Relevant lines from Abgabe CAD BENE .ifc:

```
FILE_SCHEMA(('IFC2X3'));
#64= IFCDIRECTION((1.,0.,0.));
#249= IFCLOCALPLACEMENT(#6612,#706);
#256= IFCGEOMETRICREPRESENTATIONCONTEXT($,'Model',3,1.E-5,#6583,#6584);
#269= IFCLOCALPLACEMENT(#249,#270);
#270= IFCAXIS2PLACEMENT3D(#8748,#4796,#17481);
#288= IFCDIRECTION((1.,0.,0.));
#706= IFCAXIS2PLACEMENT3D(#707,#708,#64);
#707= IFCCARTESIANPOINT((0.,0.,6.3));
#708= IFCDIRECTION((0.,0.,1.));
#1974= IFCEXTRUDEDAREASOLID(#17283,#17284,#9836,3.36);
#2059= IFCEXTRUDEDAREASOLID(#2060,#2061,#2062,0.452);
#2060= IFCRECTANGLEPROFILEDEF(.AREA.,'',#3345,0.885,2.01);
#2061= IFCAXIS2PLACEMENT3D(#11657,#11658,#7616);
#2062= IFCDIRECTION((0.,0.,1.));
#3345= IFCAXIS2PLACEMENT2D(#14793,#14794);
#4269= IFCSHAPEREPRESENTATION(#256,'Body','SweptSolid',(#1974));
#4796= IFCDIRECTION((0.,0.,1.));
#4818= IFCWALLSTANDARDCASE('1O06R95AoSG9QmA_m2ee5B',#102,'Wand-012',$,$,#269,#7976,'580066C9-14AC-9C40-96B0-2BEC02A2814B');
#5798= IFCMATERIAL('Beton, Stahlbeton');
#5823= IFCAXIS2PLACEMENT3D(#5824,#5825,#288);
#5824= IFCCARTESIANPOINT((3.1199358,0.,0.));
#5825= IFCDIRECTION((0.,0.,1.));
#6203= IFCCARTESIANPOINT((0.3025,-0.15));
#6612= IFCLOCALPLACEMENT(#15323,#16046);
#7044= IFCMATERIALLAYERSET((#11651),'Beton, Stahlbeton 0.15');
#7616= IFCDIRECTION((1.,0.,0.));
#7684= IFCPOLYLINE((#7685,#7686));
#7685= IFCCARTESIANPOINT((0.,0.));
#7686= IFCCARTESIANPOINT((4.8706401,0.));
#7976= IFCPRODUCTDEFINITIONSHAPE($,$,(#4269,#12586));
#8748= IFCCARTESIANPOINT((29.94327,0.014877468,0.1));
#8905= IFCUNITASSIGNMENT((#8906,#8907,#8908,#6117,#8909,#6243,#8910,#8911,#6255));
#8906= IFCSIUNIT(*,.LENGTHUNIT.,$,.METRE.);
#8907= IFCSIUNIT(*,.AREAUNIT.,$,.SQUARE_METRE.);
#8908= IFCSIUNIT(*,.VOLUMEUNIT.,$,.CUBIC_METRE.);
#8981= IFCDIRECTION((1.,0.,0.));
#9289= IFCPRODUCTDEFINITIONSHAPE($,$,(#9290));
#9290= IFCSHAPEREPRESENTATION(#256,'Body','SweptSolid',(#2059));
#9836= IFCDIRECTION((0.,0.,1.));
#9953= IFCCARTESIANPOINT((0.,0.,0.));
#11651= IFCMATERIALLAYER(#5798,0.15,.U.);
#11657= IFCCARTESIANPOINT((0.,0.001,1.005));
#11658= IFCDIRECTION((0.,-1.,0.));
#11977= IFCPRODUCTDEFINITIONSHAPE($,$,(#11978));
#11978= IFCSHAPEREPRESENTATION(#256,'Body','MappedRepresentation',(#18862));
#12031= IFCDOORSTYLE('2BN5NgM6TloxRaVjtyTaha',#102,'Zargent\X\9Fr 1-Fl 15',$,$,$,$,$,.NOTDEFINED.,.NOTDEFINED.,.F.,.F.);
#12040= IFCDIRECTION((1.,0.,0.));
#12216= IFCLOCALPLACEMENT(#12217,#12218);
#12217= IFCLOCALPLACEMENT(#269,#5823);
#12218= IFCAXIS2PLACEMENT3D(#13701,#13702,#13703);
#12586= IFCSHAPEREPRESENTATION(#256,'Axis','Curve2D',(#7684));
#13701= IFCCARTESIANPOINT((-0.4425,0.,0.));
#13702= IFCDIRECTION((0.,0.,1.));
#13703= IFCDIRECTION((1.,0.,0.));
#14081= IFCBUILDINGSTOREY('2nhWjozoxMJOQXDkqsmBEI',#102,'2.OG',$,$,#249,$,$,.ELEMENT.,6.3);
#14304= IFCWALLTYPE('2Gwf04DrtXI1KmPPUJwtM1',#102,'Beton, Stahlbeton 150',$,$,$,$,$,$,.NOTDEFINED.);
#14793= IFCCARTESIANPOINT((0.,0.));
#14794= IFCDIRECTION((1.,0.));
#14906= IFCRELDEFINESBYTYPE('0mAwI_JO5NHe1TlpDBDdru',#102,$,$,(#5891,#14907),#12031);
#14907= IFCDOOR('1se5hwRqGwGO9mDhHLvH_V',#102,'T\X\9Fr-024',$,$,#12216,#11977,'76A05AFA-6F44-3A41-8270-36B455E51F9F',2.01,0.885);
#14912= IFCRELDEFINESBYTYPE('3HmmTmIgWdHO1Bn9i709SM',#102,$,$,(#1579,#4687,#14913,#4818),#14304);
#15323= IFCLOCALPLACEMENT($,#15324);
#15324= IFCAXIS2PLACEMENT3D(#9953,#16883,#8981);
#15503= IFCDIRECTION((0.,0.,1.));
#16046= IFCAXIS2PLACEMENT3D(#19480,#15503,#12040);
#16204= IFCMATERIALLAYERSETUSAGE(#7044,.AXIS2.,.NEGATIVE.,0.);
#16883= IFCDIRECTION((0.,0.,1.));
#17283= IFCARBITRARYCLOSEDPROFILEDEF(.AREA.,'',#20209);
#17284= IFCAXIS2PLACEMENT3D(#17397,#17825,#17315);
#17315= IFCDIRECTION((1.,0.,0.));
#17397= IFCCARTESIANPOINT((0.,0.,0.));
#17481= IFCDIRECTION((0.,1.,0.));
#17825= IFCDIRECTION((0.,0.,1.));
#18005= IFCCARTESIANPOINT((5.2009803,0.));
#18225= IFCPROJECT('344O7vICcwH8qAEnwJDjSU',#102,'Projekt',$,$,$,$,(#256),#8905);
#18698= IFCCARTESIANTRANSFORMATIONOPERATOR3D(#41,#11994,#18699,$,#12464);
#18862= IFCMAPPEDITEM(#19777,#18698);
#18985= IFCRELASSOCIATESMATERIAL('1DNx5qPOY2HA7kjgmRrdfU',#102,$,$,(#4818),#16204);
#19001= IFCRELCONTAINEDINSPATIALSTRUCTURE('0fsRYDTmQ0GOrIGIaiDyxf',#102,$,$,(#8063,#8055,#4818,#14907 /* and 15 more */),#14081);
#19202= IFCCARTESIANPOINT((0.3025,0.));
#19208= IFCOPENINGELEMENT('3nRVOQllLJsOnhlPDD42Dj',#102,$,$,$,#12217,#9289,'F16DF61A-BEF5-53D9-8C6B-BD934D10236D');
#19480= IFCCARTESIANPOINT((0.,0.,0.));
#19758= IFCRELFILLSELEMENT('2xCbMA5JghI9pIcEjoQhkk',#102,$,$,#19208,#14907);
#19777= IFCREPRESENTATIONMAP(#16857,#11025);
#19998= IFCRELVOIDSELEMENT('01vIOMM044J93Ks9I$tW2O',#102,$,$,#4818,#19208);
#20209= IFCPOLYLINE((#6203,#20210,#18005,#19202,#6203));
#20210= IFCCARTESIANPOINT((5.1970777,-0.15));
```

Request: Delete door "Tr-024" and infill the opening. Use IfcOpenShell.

```python
import ifcopenshell
import ifcopenshell.api.feature
import ifcopenshell.api.root
import ifcopenshell.geom
import ifcopenshell.util.shape

model = ifcopenshell.open("Abgabe CAD BENE .ifc")
settings = ifcopenshell.geom.settings()


def volume(element):
    """Net volume in cubic metres, openings subtracted."""
    shape = ifcopenshell.geom.create_shape(settings, element)
    return ifcopenshell.util.shape.get_volume(shape.geometry)


door = model.by_guid("1se5hwRqGwGO9mDhHLvH_V")
opening = door.FillsVoids[0].RelatingOpeningElement
wall = opening.VoidsElements[0].RelatingBuildingElement
before = volume(wall)

ifcopenshell.api.root.remove_product(model, product=door)
ifcopenshell.api.feature.remove_feature(model, feature=opening)

after = volume(wall)

print(f"wall volume {before:.3f} -> {after:.3f} m3")

model.write("Abgabe CAD BENE _v2.ifc")
```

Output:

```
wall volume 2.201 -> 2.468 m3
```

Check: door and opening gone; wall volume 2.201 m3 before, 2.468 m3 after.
